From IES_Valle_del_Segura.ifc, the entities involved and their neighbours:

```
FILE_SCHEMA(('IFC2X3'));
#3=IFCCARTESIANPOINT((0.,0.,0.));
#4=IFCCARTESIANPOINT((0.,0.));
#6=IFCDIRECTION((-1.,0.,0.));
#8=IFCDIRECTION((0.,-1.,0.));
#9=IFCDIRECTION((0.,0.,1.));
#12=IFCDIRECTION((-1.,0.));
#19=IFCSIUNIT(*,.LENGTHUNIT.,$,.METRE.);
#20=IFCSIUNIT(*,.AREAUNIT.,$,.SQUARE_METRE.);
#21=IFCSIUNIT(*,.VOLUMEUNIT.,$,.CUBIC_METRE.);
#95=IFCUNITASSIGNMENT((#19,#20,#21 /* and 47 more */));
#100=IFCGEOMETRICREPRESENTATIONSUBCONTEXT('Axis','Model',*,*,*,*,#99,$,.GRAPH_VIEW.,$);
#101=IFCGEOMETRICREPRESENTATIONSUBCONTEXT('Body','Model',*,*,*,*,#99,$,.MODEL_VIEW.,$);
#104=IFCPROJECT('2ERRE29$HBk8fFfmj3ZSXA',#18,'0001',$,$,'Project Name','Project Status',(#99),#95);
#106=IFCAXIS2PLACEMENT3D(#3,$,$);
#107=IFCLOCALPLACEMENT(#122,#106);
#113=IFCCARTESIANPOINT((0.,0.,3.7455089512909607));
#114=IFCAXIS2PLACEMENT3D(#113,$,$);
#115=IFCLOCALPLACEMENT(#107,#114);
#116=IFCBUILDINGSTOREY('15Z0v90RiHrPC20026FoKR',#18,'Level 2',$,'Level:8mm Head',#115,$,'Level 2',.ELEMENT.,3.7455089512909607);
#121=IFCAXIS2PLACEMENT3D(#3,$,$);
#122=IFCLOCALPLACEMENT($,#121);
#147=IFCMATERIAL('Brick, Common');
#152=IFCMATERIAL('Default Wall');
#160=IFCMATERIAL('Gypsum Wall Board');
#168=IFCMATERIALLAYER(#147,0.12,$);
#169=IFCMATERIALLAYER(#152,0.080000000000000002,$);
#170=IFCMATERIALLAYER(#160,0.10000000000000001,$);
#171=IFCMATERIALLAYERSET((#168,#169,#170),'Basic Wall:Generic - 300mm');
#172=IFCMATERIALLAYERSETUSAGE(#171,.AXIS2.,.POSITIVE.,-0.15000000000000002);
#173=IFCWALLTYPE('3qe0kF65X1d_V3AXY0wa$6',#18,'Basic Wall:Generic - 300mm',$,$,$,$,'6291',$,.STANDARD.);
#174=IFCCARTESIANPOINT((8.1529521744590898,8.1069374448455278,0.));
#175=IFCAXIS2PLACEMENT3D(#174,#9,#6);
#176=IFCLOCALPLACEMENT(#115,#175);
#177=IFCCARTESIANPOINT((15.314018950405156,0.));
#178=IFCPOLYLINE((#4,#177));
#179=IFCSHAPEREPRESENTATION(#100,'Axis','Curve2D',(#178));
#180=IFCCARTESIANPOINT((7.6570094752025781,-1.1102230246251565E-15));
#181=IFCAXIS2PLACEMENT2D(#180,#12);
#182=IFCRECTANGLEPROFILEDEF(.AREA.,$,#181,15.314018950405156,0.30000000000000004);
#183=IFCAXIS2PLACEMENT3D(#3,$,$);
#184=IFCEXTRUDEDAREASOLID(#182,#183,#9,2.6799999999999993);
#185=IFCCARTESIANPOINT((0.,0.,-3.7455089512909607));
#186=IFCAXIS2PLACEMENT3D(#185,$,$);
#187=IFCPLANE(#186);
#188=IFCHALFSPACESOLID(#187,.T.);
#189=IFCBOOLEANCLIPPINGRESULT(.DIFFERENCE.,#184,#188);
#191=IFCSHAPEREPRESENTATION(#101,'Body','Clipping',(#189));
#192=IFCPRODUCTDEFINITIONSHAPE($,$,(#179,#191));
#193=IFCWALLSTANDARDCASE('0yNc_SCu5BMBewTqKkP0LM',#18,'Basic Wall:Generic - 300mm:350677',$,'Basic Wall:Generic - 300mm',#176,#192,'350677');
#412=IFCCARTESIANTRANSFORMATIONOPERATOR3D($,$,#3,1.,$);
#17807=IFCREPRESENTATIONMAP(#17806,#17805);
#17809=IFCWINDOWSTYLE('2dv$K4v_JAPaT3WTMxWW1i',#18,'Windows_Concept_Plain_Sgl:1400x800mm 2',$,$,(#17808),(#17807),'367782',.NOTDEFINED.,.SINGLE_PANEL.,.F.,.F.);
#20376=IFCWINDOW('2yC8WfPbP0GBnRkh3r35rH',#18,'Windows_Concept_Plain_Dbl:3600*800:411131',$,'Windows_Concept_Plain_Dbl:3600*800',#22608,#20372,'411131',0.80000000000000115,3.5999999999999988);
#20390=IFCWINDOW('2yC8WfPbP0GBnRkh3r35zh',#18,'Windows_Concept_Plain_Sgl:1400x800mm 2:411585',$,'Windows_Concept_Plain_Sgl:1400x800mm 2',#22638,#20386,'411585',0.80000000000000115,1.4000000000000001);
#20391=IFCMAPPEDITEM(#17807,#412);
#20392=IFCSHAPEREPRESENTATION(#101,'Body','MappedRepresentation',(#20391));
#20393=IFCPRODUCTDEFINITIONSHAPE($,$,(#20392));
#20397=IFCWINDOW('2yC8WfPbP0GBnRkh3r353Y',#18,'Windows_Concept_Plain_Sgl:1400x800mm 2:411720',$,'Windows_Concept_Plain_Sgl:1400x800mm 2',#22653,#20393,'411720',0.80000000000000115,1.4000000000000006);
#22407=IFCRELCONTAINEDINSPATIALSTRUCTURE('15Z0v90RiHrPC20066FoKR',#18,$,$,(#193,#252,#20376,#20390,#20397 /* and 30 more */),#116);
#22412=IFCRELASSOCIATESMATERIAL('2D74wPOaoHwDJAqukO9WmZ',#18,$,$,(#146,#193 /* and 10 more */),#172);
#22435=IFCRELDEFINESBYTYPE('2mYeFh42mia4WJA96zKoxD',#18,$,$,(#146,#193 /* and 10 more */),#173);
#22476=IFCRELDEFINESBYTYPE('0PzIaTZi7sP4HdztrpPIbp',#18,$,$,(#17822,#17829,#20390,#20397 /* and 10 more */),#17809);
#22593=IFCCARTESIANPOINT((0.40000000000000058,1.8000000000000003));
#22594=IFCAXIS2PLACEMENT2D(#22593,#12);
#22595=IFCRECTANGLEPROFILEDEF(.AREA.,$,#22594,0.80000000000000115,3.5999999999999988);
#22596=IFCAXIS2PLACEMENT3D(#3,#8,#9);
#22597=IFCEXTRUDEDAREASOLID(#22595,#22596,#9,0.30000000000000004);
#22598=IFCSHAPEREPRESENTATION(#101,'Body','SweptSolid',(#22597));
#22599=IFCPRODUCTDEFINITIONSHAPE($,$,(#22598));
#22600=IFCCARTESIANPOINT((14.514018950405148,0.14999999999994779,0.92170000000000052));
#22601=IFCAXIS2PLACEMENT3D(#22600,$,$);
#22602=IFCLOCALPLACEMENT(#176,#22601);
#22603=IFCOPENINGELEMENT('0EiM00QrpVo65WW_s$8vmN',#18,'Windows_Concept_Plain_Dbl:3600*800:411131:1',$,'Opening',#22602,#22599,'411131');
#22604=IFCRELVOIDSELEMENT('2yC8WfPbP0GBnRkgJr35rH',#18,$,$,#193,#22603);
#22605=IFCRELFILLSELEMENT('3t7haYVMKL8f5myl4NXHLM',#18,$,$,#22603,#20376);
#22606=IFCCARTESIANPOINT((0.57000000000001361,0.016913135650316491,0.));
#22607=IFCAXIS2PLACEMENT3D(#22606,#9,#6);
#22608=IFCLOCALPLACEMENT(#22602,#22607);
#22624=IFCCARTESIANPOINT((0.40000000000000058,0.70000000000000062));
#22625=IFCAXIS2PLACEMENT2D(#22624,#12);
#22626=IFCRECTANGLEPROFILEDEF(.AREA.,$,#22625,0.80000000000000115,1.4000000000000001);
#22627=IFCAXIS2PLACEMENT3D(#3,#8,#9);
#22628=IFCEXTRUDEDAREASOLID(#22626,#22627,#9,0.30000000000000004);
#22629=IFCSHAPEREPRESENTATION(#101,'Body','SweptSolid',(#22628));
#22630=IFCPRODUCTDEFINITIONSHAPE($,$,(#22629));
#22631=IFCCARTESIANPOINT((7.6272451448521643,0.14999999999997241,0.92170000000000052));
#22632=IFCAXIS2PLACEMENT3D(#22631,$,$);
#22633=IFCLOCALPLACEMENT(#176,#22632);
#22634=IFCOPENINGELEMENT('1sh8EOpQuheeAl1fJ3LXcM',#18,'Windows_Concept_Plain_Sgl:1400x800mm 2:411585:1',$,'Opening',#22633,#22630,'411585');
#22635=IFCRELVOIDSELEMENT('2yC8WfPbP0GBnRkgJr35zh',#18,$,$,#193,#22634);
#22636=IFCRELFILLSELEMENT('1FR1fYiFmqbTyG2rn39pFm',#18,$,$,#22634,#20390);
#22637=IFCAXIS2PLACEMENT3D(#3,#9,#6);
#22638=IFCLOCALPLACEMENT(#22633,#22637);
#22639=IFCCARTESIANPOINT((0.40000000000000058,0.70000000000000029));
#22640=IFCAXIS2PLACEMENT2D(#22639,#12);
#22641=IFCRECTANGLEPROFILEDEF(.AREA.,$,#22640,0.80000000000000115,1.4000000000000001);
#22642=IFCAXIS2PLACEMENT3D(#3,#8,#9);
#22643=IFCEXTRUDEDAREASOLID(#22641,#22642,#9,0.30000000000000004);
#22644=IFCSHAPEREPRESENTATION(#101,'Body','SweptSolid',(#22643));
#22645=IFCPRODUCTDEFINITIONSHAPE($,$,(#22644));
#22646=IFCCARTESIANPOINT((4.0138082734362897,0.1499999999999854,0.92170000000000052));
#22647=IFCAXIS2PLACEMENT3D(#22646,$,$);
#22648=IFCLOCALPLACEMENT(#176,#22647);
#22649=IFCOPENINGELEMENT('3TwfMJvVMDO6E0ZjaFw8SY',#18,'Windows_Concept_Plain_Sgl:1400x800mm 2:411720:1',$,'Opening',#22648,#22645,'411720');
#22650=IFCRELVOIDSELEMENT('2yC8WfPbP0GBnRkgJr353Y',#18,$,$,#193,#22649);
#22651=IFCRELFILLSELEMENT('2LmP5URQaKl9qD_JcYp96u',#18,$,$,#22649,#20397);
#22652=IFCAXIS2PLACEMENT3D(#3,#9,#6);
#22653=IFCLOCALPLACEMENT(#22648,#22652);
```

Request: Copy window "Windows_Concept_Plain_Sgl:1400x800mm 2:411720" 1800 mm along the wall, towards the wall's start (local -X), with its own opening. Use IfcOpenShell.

```python
import ifcopenshell
import ifcopenshell.api.feature
import ifcopenshell.api.geometry
import ifcopenshell.api.root
import ifcopenshell.geom
import ifcopenshell.util.element
import ifcopenshell.util.placement
import ifcopenshell.util.shape

model = ifcopenshell.open("IES_Valle_del_Segura.ifc")
settings = ifcopenshell.geom.settings()


def volume(element):
    """Net volume in cubic metres, openings subtracted."""
    shape = ifcopenshell.geom.create_shape(settings, element)
    return ifcopenshell.util.shape.get_volume(shape.geometry)


window = model.by_guid("2yC8WfPbP0GBnRkh3r353Y")
opening = window.FillsVoids[0].RelatingOpeningElement
wall = opening.VoidsElements[0].RelatingBuildingElement
before = volume(wall)
shift = ifcopenshell.util.placement.get_local_placement(wall.ObjectPlacement)[:3, 0] * -1.8

# copy_class copies the void relationship, type, container and properties, but no geometry.
new_opening = ifcopenshell.api.root.copy_class(model, product=opening)
new_opening.Representation = ifcopenshell.util.element.copy_deep(
    model, opening.Representation, exclude=["IfcGeometricRepresentationContext", "IfcRepresentationMap"]
)
new_opening.Name = "Windows_Concept_Plain_Sgl:1400x800mm 2"
new_opening.Tag = None
new_window = ifcopenshell.api.root.copy_class(model, product=window)
new_window.Representation = ifcopenshell.util.element.copy_deep(
    model, window.Representation, exclude=["IfcGeometricRepresentationContext", "IfcRepresentationMap"]
)
new_window.Name = "Windows_Concept_Plain_Sgl:1400x800mm 2"
new_window.Tag = None
fills = ifcopenshell.api.feature.add_filling(model, opening=new_opening, element=new_window)
fills.OwnerHistory = new_window.OwnerHistory  # required in IFC2X3

for old, new in ((opening, new_opening), (window, new_window)):
    matrix = ifcopenshell.util.placement.get_local_placement(old.ObjectPlacement)
    matrix[:3, 3] += shift
    ifcopenshell.api.geometry.edit_object_placement(model, product=new, matrix=matrix, is_si=False)

after = volume(wall)

print(f"wall volume {before:.3f} -> {after:.3f} m3")

model.write("IES_Valle_del_Segura-out.ifc")
```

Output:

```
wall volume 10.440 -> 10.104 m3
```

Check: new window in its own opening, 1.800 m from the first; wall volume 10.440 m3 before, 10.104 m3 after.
